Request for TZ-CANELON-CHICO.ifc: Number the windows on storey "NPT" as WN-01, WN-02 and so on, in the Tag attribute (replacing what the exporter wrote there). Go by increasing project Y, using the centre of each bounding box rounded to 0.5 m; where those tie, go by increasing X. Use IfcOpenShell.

First a look at what the model holds.

```python
import ifcopenshell
import ifcopenshell.util.element
import ifcopenshell.util.placement

model = ifcopenshell.open("TZ-CANELON-CHICO.ifc")
print(model.schema)
storey = next(s for s in model.by_type("IfcBuildingStorey") if s.Name == "NPT")
windows = [e for e in ifcopenshell.util.element.get_decomposition(storey) if e.is_a("IfcWindow")]
for e in sorted(windows, key=lambda e: e.id()):
    origin = ifcopenshell.util.placement.get_local_placement(e.ObjectPlacement)[:3, 3]
    print(e.id(), e.Tag, e.Name, origin.round(2) + 0.0, sep=" | ")
```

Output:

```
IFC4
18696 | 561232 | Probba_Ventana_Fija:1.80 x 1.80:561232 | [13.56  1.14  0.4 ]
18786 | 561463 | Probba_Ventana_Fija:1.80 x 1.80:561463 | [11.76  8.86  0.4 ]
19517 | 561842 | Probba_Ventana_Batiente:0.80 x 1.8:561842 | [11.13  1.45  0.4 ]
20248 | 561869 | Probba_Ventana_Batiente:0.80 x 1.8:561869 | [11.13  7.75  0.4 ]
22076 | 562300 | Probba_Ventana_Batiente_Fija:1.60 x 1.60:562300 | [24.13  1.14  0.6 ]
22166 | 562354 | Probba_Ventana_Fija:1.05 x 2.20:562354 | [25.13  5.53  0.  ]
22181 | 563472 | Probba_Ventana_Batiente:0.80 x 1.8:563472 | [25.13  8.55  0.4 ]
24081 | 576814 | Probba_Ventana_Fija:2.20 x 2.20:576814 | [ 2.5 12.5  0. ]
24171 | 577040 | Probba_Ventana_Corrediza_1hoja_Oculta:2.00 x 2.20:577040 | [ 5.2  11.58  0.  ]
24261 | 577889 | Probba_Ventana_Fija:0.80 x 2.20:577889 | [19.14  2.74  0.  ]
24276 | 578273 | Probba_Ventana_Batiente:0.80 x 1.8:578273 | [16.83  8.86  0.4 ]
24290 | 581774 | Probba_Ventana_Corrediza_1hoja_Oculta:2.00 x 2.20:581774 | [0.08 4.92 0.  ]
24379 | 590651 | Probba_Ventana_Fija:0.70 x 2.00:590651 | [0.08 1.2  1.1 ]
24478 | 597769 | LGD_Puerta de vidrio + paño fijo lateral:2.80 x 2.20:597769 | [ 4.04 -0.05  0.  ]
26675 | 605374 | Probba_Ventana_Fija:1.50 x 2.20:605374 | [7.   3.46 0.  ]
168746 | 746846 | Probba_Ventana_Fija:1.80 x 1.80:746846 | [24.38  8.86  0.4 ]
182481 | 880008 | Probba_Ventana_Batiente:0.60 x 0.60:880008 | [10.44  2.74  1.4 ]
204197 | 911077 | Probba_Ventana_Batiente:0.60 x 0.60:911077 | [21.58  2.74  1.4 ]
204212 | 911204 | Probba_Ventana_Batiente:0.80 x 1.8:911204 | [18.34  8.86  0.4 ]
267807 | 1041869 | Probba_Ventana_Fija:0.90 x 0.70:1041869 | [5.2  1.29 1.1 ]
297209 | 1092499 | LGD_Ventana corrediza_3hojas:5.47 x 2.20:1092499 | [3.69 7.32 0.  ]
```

```python
import ifcopenshell
import ifcopenshell.geom
import ifcopenshell.util.element
import ifcopenshell.util.shape

model = ifcopenshell.open("TZ-CANELON-CHICO.ifc")
settings = ifcopenshell.geom.settings()
settings.set("use-world-coords", True)


def centre(element):
    shape = ifcopenshell.geom.create_shape(settings, element)
    return ifcopenshell.util.shape.get_bbox_centroid(shape.geometry)


storey = next(s for s in model.by_type("IfcBuildingStorey") if s.Name == "NPT")
windows = [e for e in ifcopenshell.util.element.get_decomposition(storey) if e.is_a("IfcWindow")]

# Insertion points can sit at a corner or the storey origin, so sort by the geometry (in metres).
centres = {e: centre(e) for e in windows}
windows.sort(key=lambda e: (round(centres[e][1] / 0.5), centres[e][0]))

for i, e in enumerate(windows, start=1):
    number = f"WN-{i:02d}"
    e.Tag = number
    print(e.id(), number)

model.write("TZ-CANELON-CHICO_updated.ifc")
```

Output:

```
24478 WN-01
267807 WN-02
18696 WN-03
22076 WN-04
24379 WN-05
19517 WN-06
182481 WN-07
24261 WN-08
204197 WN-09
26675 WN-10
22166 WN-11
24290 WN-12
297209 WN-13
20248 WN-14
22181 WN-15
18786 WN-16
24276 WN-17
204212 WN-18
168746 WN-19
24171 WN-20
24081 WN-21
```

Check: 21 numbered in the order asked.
